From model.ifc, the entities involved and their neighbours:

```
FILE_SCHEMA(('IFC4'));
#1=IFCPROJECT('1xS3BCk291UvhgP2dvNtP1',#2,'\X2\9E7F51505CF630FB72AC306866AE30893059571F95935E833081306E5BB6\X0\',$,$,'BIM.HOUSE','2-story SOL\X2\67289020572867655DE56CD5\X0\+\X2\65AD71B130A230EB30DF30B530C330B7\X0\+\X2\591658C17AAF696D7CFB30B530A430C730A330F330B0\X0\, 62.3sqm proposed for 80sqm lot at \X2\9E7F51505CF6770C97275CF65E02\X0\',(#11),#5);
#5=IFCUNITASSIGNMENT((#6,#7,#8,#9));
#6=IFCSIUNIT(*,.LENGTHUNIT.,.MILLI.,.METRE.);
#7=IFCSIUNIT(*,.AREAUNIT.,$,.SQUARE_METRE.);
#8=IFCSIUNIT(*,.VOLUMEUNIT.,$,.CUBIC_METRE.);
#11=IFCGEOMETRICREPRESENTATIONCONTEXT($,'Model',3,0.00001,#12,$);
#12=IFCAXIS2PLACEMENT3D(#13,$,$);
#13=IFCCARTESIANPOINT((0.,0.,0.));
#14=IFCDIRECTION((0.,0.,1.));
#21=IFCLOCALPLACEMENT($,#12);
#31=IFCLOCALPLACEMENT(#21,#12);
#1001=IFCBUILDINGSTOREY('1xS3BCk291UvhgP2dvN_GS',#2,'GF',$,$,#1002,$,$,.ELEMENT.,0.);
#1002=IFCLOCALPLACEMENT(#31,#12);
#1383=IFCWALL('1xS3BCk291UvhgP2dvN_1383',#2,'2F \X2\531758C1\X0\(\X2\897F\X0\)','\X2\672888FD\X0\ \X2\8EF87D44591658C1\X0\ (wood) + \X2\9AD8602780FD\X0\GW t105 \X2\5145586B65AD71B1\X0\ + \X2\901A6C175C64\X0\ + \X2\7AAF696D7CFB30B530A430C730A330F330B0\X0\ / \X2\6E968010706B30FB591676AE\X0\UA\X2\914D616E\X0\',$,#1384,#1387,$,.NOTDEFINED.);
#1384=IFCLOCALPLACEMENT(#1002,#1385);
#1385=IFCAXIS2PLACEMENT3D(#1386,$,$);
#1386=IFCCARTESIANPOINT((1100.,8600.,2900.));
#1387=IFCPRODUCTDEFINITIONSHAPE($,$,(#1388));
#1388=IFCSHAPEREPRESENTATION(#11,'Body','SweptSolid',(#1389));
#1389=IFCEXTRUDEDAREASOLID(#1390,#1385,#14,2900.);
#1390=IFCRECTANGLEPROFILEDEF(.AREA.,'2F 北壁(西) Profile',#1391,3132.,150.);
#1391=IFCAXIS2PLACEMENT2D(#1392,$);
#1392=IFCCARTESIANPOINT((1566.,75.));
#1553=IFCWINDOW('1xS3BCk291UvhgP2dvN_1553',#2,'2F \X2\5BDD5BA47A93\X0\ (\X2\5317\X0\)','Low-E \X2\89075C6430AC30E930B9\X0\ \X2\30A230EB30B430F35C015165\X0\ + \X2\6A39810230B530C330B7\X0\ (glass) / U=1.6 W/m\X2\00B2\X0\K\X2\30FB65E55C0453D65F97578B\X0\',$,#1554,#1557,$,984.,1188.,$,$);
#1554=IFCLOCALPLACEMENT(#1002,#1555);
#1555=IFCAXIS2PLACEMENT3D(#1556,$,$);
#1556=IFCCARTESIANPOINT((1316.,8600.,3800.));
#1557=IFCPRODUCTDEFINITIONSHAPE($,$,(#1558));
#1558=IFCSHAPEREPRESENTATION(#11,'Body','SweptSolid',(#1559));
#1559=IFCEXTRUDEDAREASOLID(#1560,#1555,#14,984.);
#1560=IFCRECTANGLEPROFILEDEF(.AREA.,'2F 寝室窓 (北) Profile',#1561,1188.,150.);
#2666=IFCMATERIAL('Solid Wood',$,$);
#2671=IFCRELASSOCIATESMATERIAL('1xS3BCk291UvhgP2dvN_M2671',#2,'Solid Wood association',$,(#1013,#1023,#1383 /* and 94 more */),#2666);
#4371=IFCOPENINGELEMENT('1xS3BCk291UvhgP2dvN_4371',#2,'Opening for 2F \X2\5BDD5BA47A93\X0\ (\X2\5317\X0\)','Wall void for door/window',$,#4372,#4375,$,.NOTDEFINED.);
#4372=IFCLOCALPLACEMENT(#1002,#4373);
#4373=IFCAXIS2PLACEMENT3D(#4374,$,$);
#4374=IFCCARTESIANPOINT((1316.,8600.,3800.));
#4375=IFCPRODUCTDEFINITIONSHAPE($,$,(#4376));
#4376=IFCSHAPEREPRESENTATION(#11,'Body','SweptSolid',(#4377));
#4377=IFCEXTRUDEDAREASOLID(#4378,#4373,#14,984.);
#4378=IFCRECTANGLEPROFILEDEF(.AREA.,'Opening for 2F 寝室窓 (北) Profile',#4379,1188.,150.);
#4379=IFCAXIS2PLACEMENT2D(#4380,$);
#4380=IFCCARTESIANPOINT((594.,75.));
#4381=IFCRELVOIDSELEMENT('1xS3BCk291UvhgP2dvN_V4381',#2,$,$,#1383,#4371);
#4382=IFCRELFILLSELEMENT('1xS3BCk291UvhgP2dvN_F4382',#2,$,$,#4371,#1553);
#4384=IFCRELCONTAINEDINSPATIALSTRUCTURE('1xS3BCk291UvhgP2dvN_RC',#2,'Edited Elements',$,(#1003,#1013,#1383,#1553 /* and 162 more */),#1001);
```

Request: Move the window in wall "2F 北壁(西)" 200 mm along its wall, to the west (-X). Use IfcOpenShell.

```python
import ifcopenshell
import ifcopenshell.api.geometry
import ifcopenshell.util.placement
import ifcopenshell.util.unit

model = ifcopenshell.open("model.ifc")
unit_scale = ifcopenshell.util.unit.calculate_unit_scale(model)

window = model.by_id(1553)
opening = window.FillsVoids[0].RelatingOpeningElement
wall = opening.VoidsElements[0].RelatingBuildingElement

wall_matrix = ifcopenshell.util.placement.get_local_placement(wall.ObjectPlacement)
shift = wall_matrix[:3, 0] * -0.2 / unit_scale
before = ifcopenshell.util.placement.get_local_placement(window.ObjectPlacement)[:3, 3].copy()

# The window is not placed relative to its opening, so move both.
for product in (opening, window):
    matrix = ifcopenshell.util.placement.get_local_placement(product.ObjectPlacement)
    matrix[:3, 3] += shift
    ifcopenshell.api.geometry.edit_object_placement(model, product=product, matrix=matrix, is_si=False)

after = ifcopenshell.util.placement.get_local_placement(window.ObjectPlacement)[:3, 3]
print("window moved by", (after - before).round(3) + 0.0)

model.write("model_edited.ifc")
```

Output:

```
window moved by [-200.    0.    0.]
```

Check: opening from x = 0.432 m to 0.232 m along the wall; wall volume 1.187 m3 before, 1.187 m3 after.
